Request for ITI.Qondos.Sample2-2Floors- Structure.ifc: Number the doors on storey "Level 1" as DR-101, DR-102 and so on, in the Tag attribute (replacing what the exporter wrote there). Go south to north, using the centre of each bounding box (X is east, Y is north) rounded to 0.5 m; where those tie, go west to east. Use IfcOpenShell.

First a look at what the model holds.

```python
import ifcopenshell
import ifcopenshell.util.element
import ifcopenshell.util.placement

model = ifcopenshell.open("ITI.Qondos.Sample2-2Floors- Structure.ifc")
print(model.schema)
storey = next(s for s in model.by_type("IfcBuildingStorey") if s.Name == "Level 1")
doors = [e for e in ifcopenshell.util.element.get_decomposition(storey) if e.is_a("IfcDoor")]
for e in sorted(doors, key=lambda e: e.id()):
    origin = ifcopenshell.util.placement.get_local_placement(e.ObjectPlacement)[:3, 3]
    print(e.id(), e.Tag, e.Name, origin.round(2) + 0.0, sep=" | ")
```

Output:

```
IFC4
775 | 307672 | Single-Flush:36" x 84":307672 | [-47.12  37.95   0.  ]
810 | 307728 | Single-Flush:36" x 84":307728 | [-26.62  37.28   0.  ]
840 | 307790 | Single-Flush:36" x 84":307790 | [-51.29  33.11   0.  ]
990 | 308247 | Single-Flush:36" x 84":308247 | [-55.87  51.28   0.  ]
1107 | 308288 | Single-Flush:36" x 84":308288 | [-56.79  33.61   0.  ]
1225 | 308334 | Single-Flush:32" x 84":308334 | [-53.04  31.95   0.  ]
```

```python
import ifcopenshell
import ifcopenshell.geom
import ifcopenshell.util.element
import ifcopenshell.util.shape

model = ifcopenshell.open("ITI.Qondos.Sample2-2Floors- Structure.ifc")
settings = ifcopenshell.geom.settings()
settings.set("use-world-coords", True)


def centre(element):
    shape = ifcopenshell.geom.create_shape(settings, element)
    return ifcopenshell.util.shape.get_bbox_centroid(shape.geometry)


storey = next(s for s in model.by_type("IfcBuildingStorey") if s.Name == "Level 1")
doors = [e for e in ifcopenshell.util.element.get_decomposition(storey) if e.is_a("IfcDoor")]

# Insertion points can sit at a corner or the storey origin, so sort by the geometry (in metres).
centres = {e: centre(e) for e in doors}
doors.sort(key=lambda e: (round(centres[e][1] / 0.5), centres[e][0]))

for i, e in enumerate(doors, start=1):
    number = f"DR-1{i:02d}"
    e.Tag = number
    print(e.id(), number)

model.write("ITI.Qondos.Sample2-2Floors- Structure_rev.ifc")
```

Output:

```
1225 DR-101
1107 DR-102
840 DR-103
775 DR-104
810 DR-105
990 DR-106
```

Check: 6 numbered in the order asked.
